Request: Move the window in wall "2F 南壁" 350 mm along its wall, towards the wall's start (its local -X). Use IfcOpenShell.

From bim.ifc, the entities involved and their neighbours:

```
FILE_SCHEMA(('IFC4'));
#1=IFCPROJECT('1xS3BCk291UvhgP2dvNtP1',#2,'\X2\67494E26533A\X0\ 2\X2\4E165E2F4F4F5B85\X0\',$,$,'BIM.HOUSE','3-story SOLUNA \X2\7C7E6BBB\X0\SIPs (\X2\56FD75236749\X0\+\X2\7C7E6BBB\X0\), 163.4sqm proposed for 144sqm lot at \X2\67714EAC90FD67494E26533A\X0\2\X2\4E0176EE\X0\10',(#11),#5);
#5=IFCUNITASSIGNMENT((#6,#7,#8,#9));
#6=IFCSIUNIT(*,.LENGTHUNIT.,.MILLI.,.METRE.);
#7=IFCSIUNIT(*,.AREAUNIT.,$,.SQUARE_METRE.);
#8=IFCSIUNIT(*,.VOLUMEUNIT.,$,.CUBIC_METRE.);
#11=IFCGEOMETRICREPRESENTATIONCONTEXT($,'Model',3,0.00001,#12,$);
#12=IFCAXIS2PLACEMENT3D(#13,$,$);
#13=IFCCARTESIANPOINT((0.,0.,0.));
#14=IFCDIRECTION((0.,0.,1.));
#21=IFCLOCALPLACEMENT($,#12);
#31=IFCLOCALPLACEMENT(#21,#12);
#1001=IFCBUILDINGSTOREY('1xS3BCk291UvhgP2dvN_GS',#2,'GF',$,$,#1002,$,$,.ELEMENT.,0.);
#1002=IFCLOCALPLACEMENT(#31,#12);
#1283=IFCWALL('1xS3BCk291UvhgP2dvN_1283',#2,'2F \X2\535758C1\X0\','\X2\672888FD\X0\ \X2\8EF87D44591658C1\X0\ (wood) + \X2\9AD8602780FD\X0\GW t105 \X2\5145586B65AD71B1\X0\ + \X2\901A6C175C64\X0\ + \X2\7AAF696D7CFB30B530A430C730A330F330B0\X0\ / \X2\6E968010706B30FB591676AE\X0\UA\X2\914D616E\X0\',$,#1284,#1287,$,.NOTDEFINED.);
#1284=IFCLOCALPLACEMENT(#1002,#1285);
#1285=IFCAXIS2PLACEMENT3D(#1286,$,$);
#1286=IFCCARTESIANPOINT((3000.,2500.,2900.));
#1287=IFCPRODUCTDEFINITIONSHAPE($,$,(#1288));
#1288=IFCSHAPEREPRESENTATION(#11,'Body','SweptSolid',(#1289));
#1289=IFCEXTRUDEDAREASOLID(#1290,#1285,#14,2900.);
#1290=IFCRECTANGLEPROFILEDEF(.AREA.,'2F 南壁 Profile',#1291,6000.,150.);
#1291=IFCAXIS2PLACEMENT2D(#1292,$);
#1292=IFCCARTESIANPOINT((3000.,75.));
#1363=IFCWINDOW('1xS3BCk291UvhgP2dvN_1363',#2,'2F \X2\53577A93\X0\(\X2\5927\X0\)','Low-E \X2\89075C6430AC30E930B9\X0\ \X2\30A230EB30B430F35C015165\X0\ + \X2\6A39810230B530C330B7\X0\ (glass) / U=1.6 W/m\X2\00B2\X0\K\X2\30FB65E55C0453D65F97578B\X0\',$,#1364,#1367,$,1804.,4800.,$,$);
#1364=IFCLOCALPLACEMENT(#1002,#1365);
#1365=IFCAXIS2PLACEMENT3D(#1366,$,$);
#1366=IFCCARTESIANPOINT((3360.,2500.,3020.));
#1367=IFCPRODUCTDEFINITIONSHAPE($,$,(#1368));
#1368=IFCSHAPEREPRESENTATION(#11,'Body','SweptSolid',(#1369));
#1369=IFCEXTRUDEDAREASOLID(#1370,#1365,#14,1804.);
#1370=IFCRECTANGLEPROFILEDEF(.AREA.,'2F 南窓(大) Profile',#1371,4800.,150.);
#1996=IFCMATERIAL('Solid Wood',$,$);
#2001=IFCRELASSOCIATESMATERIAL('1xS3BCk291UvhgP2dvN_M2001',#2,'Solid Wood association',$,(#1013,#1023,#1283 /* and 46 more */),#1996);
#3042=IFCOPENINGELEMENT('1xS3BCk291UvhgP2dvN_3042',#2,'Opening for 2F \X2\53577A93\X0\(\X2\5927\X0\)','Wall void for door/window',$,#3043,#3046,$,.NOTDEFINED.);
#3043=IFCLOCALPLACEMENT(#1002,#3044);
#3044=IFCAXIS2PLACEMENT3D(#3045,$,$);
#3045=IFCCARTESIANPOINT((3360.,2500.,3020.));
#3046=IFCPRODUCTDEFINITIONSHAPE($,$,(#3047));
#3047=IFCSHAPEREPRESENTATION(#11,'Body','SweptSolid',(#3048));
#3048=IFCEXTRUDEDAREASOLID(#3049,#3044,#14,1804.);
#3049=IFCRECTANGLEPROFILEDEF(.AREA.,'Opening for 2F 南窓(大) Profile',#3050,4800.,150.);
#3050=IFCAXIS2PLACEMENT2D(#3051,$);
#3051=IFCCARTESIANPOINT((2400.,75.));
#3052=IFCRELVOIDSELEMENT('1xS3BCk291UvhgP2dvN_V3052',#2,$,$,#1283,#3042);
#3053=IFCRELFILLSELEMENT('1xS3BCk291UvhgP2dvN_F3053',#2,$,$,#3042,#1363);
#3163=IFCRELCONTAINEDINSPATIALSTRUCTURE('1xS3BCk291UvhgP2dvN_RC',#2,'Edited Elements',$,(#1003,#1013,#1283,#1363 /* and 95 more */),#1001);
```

```python
import ifcopenshell
import ifcopenshell.api.geometry
import ifcopenshell.util.placement
import ifcopenshell.util.unit

model = ifcopenshell.open("bim.ifc")
unit_scale = ifcopenshell.util.unit.calculate_unit_scale(model)

window = model.by_guid("1xS3BCk291UvhgP2dvN_1363")
opening = window.FillsVoids[0].RelatingOpeningElement
wall = opening.VoidsElements[0].RelatingBuildingElement

wall_matrix = ifcopenshell.util.placement.get_local_placement(wall.ObjectPlacement)
shift = wall_matrix[:3, 0] * -0.35 / unit_scale
before = ifcopenshell.util.placement.get_local_placement(window.ObjectPlacement)[:3, 3].copy()

# The window is not placed relative to its opening, so move both.
for product in (opening, window):
    matrix = ifcopenshell.util.placement.get_local_placement(product.ObjectPlacement)
    matrix[:3, 3] += shift
    ifcopenshell.api.geometry.edit_object_placement(model, product=product, matrix=matrix, is_si=False)

after = ifcopenshell.util.placement.get_local_placement(window.ObjectPlacement)[:3, 3]
print("window moved by", (after - before).round(3) + 0.0)

model.write("bim_rev.ifc")
```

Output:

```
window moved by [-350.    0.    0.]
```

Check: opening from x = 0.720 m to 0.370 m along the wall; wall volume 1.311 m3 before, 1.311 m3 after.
